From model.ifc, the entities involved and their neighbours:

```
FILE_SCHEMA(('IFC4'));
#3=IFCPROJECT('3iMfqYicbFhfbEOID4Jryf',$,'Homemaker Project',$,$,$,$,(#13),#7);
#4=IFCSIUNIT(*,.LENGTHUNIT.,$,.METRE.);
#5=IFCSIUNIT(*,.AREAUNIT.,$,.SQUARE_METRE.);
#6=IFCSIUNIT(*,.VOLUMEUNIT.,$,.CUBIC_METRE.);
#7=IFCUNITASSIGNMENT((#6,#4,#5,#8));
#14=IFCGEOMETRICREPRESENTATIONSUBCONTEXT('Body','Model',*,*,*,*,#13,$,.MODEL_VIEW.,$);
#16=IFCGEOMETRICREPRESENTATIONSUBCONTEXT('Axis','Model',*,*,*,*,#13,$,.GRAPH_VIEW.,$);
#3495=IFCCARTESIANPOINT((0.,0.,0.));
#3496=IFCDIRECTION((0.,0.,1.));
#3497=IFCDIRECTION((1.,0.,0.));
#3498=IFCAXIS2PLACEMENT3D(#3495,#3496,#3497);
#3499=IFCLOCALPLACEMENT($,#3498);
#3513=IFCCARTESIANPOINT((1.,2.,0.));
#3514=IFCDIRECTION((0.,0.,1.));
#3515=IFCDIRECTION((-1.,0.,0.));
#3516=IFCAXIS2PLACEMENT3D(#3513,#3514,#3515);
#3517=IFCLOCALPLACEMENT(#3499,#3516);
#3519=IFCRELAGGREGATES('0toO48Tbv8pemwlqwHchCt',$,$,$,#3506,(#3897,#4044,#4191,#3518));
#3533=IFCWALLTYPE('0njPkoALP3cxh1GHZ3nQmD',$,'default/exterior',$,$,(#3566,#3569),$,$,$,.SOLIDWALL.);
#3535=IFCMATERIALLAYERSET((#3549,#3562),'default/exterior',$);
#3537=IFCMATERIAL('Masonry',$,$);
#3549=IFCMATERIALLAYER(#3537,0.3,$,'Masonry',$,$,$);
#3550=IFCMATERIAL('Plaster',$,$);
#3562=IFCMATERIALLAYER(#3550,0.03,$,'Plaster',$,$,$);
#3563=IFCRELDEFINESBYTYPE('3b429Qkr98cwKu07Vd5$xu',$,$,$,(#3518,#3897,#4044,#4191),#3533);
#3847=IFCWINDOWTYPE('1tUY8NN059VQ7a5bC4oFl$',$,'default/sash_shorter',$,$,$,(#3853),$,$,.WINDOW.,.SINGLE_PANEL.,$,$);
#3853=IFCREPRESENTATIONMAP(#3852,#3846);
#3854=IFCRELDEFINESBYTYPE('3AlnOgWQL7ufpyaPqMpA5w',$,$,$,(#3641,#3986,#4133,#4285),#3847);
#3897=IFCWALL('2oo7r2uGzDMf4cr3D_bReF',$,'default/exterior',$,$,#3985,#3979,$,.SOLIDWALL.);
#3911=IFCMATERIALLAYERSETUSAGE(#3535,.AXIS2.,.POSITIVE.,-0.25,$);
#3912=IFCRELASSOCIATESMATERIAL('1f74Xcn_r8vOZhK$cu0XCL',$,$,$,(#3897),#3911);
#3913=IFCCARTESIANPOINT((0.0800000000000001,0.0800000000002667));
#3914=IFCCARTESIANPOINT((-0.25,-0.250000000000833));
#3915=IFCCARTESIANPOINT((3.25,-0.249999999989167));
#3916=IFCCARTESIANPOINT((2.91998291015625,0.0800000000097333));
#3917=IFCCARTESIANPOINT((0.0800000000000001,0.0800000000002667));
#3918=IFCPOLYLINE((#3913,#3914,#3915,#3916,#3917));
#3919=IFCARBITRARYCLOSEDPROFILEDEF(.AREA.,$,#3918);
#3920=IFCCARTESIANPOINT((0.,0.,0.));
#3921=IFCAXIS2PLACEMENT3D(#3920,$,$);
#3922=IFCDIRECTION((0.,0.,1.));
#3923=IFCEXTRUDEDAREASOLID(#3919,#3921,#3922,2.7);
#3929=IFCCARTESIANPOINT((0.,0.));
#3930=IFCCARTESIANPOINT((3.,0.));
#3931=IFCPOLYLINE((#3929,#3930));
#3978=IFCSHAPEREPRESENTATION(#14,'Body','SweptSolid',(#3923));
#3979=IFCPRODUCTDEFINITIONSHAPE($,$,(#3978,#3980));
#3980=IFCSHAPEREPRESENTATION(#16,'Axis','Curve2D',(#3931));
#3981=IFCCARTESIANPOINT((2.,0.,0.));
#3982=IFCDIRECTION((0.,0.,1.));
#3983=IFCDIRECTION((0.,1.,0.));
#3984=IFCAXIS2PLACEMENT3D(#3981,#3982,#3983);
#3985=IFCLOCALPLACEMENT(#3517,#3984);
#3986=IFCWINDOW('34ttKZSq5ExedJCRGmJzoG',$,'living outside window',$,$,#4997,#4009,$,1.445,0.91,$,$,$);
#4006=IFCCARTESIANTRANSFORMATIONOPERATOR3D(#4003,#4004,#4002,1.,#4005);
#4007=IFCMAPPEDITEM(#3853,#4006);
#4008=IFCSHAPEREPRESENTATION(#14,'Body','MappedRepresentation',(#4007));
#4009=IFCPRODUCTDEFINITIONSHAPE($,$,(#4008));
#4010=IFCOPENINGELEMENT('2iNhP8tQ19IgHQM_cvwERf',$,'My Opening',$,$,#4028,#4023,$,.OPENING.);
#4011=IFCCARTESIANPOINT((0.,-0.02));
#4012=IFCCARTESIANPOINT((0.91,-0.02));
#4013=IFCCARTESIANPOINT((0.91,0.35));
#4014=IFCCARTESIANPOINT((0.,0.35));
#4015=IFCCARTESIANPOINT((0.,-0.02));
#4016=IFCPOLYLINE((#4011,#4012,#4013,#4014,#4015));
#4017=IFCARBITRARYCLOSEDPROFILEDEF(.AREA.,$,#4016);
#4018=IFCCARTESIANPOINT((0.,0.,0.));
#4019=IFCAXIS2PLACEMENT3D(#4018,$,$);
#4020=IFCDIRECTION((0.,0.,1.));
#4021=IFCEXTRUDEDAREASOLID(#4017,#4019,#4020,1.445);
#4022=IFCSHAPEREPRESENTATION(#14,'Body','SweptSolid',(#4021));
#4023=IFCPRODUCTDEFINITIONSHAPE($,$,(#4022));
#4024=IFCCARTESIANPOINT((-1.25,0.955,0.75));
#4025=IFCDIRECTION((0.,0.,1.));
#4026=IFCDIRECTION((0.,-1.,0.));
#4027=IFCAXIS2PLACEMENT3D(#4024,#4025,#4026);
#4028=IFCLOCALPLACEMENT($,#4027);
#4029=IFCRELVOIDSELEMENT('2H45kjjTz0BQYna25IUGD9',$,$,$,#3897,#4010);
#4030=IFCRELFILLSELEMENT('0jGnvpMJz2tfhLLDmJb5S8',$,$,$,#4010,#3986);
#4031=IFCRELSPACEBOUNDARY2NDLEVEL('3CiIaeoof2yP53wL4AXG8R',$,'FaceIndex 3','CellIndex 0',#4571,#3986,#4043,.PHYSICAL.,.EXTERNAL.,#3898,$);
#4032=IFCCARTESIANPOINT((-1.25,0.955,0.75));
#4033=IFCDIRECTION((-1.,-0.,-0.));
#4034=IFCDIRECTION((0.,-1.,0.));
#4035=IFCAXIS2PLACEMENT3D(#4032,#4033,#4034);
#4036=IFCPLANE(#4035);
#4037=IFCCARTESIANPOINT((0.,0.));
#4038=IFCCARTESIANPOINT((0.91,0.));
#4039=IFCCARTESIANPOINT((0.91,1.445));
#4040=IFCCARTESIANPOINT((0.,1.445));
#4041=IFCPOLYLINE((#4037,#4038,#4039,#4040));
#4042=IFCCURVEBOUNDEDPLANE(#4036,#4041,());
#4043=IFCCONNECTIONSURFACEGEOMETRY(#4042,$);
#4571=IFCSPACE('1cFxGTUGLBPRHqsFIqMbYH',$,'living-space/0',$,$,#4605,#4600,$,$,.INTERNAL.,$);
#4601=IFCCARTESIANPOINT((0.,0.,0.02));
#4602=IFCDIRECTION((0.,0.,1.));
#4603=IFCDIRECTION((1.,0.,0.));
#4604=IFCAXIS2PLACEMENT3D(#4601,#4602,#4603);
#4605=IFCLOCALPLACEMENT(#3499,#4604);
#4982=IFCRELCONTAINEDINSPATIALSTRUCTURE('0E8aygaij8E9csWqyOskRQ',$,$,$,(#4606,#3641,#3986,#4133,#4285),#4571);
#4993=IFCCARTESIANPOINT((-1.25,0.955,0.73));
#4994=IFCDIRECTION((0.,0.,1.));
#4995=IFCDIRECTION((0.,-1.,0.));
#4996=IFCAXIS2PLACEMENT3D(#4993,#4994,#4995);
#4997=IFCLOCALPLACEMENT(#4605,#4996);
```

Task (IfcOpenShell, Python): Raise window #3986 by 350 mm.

```python
import numpy as np
import ifcopenshell
import ifcopenshell.api.geometry
import ifcopenshell.util.placement
import ifcopenshell.util.unit

model = ifcopenshell.open("model.ifc")
unit_scale = ifcopenshell.util.unit.calculate_unit_scale(model)

window = model.by_guid("34ttKZSq5ExedJCRGmJzoG")
opening = window.FillsVoids[0].RelatingOpeningElement
dz = 0.35 / unit_scale

shift = np.array([0.0, 0.0, dz])
# The window is not placed relative to its opening, so move both.
for product in (opening, window):
    matrix = ifcopenshell.util.placement.get_local_placement(product.ObjectPlacement)
    matrix[:3, 3] += shift
    ifcopenshell.api.geometry.edit_object_placement(model, product=product, matrix=matrix, is_si=False)

# Space boundary surfaces are stored in each space's coordinates; move them too.
for rel in window.ProvidesBoundaries:
    if not rel.ConnectionGeometry:
        continue
    surface = rel.ConnectionGeometry.SurfaceOnRelatingElement.BasisSurface
    space_matrix = ifcopenshell.util.placement.get_local_placement(rel.RelatingSpace.ObjectPlacement)
    point = np.array(surface.Position.Location.Coordinates) + space_matrix[:3, :3].T @ shift
    surface.Position = model.createIfcAxis2Placement3D(
        model.createIfcCartesianPoint(point.tolist()), surface.Position.Axis, surface.Position.RefDirection
    )

print(f"moved by {dz * unit_scale:+.3f} m")

model.write("model-out.ifc")
```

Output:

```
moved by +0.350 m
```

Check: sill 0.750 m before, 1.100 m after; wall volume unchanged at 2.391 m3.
